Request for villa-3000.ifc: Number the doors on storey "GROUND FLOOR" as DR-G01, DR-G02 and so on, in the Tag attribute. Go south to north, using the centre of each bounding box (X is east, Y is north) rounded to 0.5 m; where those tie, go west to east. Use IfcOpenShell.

First a look at what the model holds.

```python
import ifcopenshell
import ifcopenshell.util.element
import ifcopenshell.util.placement

model = ifcopenshell.open("villa-3000.ifc")
print(model.schema)
storey = next(s for s in model.by_type("IfcBuildingStorey") if s.Name == "GROUND FLOOR")
doors = [e for e in ifcopenshell.util.element.get_decomposition(storey) if e.is_a("IfcDoor")]
for e in sorted(doors, key=lambda e: e.id()):
    origin = ifcopenshell.util.placement.get_local_placement(e.ObjectPlacement)[:3, 3]
    print(e.id(), e.Tag, e.Name, origin.round(2) + 0.0, sep=" | ")
```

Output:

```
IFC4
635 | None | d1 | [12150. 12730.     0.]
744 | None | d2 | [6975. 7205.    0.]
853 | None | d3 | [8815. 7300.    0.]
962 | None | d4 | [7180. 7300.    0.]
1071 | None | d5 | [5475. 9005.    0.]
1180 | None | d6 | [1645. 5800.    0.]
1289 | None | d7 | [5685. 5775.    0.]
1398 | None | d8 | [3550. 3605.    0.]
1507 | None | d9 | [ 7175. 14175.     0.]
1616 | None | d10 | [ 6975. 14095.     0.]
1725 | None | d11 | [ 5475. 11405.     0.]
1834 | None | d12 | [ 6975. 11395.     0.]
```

```python
import ifcopenshell
import ifcopenshell.geom
import ifcopenshell.util.element
import ifcopenshell.util.shape

model = ifcopenshell.open("villa-3000.ifc")
settings = ifcopenshell.geom.settings()
settings.set("use-world-coords", True)


def centre(element):
    shape = ifcopenshell.geom.create_shape(settings, element)
    return ifcopenshell.util.shape.get_bbox_centroid(shape.geometry)


storey = next(s for s in model.by_type("IfcBuildingStorey") if s.Name == "GROUND FLOOR")
doors = [e for e in ifcopenshell.util.element.get_decomposition(storey) if e.is_a("IfcDoor")]

# Insertion points can sit at a corner or the storey origin, so sort by the geometry (in metres).
centres = {e: centre(e) for e in doors}
doors.sort(key=lambda e: (round(centres[e][1] / 0.5), centres[e][0]))

for i, e in enumerate(doors, start=1):
    number = f"DR-G{i:02d}"
    e.Tag = number
    print(e.id(), number)

model.write("villa-3000_rev.ifc")
```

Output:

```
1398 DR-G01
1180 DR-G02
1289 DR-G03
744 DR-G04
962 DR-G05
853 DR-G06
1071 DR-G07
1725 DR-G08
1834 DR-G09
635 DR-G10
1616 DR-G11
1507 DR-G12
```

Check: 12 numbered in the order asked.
